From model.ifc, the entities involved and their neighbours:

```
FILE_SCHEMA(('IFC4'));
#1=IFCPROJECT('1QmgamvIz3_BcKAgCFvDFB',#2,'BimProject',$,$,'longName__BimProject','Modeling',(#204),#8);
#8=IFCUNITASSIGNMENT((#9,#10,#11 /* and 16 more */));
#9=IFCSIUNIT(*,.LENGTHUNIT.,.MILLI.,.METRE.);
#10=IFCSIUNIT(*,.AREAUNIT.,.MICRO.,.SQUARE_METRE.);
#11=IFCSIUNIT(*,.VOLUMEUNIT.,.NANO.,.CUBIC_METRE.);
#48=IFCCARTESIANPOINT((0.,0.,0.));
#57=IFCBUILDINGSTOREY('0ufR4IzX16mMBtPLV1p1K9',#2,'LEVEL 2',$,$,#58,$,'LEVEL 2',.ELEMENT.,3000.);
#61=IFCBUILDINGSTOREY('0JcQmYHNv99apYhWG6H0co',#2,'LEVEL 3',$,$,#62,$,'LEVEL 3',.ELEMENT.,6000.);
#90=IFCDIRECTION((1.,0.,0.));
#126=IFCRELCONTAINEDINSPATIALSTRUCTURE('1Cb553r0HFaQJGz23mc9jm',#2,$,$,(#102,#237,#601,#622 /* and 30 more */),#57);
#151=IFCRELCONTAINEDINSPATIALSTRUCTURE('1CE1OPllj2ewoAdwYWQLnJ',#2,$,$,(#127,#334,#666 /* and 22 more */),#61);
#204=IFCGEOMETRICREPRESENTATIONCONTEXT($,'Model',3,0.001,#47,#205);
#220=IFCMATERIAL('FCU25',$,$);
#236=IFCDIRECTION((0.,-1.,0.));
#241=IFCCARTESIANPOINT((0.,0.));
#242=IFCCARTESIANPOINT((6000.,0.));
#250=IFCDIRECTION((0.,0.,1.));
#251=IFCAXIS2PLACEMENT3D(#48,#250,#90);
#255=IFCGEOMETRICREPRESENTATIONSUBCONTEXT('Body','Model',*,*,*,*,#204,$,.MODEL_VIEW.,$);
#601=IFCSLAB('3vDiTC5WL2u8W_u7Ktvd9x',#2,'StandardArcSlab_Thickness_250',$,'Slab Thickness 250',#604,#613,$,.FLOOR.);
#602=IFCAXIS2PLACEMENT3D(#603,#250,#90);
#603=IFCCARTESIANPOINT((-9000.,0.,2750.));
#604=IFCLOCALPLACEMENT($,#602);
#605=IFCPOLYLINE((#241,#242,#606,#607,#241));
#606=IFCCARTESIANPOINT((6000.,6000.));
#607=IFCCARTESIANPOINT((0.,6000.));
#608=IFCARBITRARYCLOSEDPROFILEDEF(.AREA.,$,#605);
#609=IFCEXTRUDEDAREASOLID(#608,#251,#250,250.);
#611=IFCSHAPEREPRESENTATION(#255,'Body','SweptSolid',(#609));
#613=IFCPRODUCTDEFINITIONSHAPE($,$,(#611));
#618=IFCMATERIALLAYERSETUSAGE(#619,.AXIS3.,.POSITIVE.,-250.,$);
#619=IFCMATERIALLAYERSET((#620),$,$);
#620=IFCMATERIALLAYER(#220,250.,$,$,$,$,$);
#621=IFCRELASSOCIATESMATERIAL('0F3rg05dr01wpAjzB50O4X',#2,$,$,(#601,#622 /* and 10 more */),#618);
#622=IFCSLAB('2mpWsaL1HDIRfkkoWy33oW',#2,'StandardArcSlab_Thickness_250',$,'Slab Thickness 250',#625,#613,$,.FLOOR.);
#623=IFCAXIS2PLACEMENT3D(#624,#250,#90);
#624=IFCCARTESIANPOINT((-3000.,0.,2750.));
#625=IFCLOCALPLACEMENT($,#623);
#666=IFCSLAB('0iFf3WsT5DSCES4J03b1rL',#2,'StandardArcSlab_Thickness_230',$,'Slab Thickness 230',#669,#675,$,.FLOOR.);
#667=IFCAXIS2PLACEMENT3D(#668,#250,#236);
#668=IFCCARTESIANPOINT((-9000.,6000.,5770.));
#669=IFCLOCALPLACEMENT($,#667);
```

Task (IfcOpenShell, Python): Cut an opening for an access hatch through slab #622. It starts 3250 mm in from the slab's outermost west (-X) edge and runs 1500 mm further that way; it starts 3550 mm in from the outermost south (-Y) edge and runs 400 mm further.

```python
import numpy as np
import ifcopenshell
import ifcopenshell.api.feature
import ifcopenshell.api.geometry
import ifcopenshell.api.root
import ifcopenshell.geom
import ifcopenshell.util.placement
import ifcopenshell.util.representation
import ifcopenshell.util.shape
import ifcopenshell.util.unit

model = ifcopenshell.open("model.ifc")
unit_scale = ifcopenshell.util.unit.calculate_unit_scale(model)
settings = ifcopenshell.geom.settings()


def volume(element):
    """Net volume in cubic metres, openings subtracted."""
    shape = ifcopenshell.geom.create_shape(settings, element)
    return ifcopenshell.util.shape.get_volume(shape.geometry)


slab = model.by_guid("2mpWsaL1HDIRfkkoWy33oW")
before = volume(slab)

# Extent in the slab's own axes, in metres. The edges named are its -X and -Y sides.
slab_shape = ifcopenshell.geom.create_shape(settings, slab)
vertices = ifcopenshell.util.shape.get_vertices(slab_shape.geometry)
x_min, y_min, bottom = vertices.min(axis=0)
top = vertices[:, 2].max()

opening = ifcopenshell.api.root.create_entity(model, ifc_class="IfcOpeningElement", name="Access hatch opening", predefined_type="OPENING")
context = ifcopenshell.util.representation.get_context(model, "Model", "Body", "MODEL_VIEW")
width, depth = 1.5, 0.4
outline = [(0.0, 0.0), (width, 0.0), (width, depth), (0.0, depth), (0.0, 0.0)]
# Overshoot both faces by 50 mm so the cut is clean.
shape = ifcopenshell.api.geometry.add_slab_representation(
    model, context=context, depth=top - bottom + 0.1, polyline=outline
)
ifcopenshell.api.geometry.assign_representation(model, product=opening, representation=shape)

matrix = ifcopenshell.util.placement.get_local_placement(slab.ObjectPlacement)
matrix[:, 3] = matrix @ np.append(np.array([x_min + 3.25, y_min + 3.55, bottom - 0.05]) / unit_scale, 1.0)
ifcopenshell.api.geometry.edit_object_placement(model, product=opening, matrix=matrix, is_si=False)
ifcopenshell.api.feature.add_feature(model, feature=opening, element=slab)

after = volume(slab)

print(f"slab volume {before:.3f} -> {after:.3f} m3")

model.write("model_v2.ifc")
```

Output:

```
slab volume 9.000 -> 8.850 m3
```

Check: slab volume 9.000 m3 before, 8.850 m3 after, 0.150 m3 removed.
